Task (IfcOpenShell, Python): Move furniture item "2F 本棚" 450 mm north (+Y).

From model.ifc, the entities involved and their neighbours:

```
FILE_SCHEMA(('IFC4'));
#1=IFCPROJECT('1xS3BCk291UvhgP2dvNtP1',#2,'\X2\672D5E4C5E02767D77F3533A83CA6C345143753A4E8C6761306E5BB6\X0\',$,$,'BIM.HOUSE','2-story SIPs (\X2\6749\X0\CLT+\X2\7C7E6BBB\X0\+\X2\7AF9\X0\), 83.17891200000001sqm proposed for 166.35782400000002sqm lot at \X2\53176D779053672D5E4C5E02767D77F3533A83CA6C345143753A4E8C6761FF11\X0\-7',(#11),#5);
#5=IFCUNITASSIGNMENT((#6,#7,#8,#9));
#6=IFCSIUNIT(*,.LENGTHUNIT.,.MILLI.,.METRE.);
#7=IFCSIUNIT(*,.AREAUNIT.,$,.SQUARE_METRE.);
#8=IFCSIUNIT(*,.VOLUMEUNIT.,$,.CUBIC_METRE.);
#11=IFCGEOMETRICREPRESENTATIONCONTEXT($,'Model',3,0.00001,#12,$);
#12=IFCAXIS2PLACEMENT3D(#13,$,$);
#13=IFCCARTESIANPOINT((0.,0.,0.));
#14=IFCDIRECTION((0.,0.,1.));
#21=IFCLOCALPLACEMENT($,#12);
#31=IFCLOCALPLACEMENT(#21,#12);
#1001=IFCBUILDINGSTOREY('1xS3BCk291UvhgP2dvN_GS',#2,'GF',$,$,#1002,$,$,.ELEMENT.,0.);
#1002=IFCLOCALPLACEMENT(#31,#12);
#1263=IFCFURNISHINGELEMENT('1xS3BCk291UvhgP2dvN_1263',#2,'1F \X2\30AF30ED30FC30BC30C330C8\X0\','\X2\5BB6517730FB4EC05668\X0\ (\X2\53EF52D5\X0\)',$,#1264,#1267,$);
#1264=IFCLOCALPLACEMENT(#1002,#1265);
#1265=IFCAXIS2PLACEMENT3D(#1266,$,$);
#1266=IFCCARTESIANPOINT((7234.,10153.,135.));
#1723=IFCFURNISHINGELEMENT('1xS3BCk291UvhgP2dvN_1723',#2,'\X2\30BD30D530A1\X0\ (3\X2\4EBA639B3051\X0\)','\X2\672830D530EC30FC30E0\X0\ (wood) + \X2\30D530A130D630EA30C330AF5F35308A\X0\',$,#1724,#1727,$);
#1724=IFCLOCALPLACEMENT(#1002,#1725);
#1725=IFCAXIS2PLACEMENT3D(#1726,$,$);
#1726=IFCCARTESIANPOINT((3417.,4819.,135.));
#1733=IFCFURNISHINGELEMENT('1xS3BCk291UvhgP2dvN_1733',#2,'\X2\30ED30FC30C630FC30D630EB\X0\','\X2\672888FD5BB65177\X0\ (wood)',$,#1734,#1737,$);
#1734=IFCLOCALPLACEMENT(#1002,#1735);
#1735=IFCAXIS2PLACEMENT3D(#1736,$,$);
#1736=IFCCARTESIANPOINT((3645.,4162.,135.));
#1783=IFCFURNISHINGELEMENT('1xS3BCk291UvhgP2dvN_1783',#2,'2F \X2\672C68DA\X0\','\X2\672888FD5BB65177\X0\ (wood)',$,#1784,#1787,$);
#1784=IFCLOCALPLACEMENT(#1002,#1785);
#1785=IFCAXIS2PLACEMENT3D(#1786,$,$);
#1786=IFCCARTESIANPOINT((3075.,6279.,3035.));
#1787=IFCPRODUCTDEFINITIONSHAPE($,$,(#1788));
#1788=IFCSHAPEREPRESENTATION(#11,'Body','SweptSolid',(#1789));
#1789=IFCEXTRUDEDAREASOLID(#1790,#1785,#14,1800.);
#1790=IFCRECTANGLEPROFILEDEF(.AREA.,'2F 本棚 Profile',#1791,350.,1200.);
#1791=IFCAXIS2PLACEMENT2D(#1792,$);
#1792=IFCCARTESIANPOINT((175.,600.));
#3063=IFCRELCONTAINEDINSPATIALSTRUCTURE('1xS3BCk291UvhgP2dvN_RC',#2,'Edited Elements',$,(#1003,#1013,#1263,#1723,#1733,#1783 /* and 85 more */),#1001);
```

```python
import ifcopenshell
import ifcopenshell.api.geometry
import ifcopenshell.util.placement
import ifcopenshell.util.unit

model = ifcopenshell.open("model.ifc")
unit_scale = ifcopenshell.util.unit.calculate_unit_scale(model)

item = model.by_guid("1xS3BCk291UvhgP2dvN_1783")
matrix = ifcopenshell.util.placement.get_local_placement(item.ObjectPlacement)
matrix[1, 3] += 0.45 / unit_scale
ifcopenshell.api.geometry.edit_object_placement(model, product=item, matrix=matrix, is_si=False)

print(ifcopenshell.util.placement.get_local_placement(item.ObjectPlacement).round(3) + 0.0)

model.write("model_rev.ifc")
```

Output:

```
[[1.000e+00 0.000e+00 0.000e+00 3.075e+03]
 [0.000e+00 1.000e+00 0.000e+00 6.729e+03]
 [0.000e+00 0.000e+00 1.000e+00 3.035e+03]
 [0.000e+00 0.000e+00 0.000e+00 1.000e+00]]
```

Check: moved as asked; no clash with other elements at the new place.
